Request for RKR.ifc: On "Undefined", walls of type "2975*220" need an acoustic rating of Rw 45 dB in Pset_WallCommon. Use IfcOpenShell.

First a look at what the model holds.

```python
import ifcopenshell
import ifcopenshell.util.element

model = ifcopenshell.open("RKR.ifc")
print(model.schema)
storey = next(s for s in model.by_type("IfcBuildingStorey") if s.Name == "Undefined")
walls = [e for e in ifcopenshell.util.element.get_decomposition(storey) if e.is_a("IfcWall")]
seen = {}
for e in walls:
    element_type = ifcopenshell.util.element.get_type(e)
    key = (element_type.Name if element_type != e and element_type else None, ifcopenshell.util.element.get_pset(e, "Pset_WallCommon", "AcousticRating"))
    seen[key] = seen.get(key, 0) + 1
for (name, value), count in sorted(seen.items(), key=str):
    print(count, "x", name, "|", value)
```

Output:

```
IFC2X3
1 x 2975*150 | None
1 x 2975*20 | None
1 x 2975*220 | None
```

```python
import ifcopenshell
import ifcopenshell.api.pset
import ifcopenshell.util.element

model = ifcopenshell.open("RKR.ifc")

storey = next(s for s in model.by_type("IfcBuildingStorey") if s.Name == "Undefined")
walls = [e for e in ifcopenshell.util.element.get_decomposition(storey) if e.is_a("IfcWall")]

count = 0
for e in walls:
    element_type = ifcopenshell.util.element.get_type(e)
    if element_type in (None, e) or element_type.Name != "2975*220":
        continue
    # add_pset returns the element's existing set when there is one.
    pset = ifcopenshell.api.pset.add_pset(model, product=e, name="Pset_WallCommon")
    ifcopenshell.api.pset.edit_pset(model, pset=pset, properties={"AcousticRating": "Rw 45 dB"})
    count += 1

print(count, "walls updated")

model.write("RKR_v2.ifc")
```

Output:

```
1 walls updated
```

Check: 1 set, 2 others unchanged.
